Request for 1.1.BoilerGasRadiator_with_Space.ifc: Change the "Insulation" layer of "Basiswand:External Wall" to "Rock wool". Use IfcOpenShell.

First a look at what the model holds.

```python
import ifcopenshell
import ifcopenshell.util.element

model = ifcopenshell.open("1.1.BoilerGasRadiator_with_Space.ifc")
print(model.schema)
for layer_set in model.by_type("IfcMaterialLayerSet"):
    if layer_set.LayerSetName == "Basiswand:External Wall":
        for layer in layer_set.MaterialLayers:
            print(layer.id(), layer.Material and layer.Material.Name, layer.LayerThickness, sep=" | ")
        print(len(ifcopenshell.util.element.get_elements_by_material(model, layer_set)), "elements and types use it")
print(sorted(m.Name for m in model.by_type("IfcMaterial") if m.Name)[:60])
```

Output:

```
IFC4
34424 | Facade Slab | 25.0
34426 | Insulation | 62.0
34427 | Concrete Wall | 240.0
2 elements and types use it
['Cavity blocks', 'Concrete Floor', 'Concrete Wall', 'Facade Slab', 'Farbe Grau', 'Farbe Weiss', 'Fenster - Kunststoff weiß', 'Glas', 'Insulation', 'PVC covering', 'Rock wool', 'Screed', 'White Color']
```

```python
import ifcopenshell
import ifcopenshell.api.material

model = ifcopenshell.open("1.1.BoilerGasRadiator_with_Space.ifc")

layer_set = next(s for s in model.by_type("IfcMaterialLayerSet") if s.LayerSetName == "Basiswand:External Wall")
layer = next(l for l in layer_set.MaterialLayers if l.Material and l.Material.Name == "Insulation")
material = next(m for m in model.by_type("IfcMaterial") if m.Name == "Rock wool")

# Point this one layer at the other material; renaming the old one would change it everywhere.
ifcopenshell.api.material.edit_layer(model, layer=layer, attributes={}, material=material)

print([l.Material.Name if l.Material else None for l in layer_set.MaterialLayers])

model.write("1.1.BoilerGasRadiator_with_Space_rev.ifc")
```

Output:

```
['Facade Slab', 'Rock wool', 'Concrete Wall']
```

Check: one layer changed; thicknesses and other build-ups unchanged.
